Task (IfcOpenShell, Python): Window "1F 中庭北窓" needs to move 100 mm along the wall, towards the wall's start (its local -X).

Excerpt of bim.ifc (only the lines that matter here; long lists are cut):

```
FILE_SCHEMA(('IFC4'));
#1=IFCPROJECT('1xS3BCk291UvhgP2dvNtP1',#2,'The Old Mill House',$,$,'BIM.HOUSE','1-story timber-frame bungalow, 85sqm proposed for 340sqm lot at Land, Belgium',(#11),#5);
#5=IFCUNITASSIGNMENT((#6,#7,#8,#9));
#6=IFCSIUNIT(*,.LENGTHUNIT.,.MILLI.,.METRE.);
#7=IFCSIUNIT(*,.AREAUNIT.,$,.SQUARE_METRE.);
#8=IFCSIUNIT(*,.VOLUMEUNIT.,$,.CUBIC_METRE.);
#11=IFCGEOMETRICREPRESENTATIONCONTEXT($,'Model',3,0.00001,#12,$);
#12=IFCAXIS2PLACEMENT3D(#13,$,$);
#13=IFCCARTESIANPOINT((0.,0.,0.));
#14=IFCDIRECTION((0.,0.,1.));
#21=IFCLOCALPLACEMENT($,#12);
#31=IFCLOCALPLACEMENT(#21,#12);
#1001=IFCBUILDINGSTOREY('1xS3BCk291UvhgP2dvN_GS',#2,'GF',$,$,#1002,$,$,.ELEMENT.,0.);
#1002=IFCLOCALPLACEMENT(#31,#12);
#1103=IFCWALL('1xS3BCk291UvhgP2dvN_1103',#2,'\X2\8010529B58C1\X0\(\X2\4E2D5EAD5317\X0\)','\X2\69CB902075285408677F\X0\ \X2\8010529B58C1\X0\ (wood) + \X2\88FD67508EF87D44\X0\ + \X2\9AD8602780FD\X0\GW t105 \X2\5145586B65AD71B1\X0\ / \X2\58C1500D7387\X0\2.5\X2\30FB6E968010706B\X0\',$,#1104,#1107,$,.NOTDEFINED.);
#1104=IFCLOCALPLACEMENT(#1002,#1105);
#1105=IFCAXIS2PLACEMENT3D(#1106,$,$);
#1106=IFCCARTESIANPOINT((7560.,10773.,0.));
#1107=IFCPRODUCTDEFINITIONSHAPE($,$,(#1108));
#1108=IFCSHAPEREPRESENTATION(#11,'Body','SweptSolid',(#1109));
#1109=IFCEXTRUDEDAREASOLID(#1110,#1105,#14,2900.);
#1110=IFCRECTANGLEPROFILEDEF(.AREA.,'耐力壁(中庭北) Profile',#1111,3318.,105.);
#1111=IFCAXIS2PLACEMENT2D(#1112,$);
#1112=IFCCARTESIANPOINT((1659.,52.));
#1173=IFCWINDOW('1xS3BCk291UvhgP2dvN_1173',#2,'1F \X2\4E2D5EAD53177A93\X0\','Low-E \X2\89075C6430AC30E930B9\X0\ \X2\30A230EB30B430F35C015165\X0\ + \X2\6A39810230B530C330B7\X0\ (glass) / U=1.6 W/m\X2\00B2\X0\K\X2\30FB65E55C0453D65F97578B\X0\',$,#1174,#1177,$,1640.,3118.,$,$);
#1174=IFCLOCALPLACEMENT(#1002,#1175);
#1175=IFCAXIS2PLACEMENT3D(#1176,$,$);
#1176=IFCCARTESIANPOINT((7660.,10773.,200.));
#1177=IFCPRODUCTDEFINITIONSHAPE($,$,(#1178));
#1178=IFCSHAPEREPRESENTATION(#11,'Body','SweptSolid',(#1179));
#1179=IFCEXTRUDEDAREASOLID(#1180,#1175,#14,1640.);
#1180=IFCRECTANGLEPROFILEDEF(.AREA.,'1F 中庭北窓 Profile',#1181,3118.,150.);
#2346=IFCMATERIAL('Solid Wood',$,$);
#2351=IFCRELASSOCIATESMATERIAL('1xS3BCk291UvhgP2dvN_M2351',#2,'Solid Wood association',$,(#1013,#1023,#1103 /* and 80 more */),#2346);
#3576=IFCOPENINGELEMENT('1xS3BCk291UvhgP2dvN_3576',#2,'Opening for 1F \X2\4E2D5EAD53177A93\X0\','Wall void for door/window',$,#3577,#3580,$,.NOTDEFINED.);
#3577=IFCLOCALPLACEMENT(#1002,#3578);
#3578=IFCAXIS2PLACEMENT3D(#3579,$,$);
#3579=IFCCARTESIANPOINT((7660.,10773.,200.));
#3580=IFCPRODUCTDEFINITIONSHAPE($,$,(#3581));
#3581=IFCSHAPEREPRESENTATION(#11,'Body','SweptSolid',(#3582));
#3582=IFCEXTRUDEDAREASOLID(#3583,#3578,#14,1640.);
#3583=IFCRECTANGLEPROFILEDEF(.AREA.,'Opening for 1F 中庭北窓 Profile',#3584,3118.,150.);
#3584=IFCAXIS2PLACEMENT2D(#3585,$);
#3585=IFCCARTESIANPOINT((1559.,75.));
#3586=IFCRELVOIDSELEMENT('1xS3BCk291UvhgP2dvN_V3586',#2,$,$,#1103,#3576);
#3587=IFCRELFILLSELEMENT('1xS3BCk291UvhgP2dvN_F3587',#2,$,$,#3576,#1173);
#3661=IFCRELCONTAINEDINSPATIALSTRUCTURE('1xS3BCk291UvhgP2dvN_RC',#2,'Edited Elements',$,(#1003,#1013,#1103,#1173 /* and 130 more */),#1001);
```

```python
import ifcopenshell
import ifcopenshell.api.geometry
import ifcopenshell.util.placement
import ifcopenshell.util.unit

model = ifcopenshell.open("bim.ifc")
unit_scale = ifcopenshell.util.unit.calculate_unit_scale(model)

window = model.by_id(1173)
opening = window.FillsVoids[0].RelatingOpeningElement
wall = opening.VoidsElements[0].RelatingBuildingElement

wall_matrix = ifcopenshell.util.placement.get_local_placement(wall.ObjectPlacement)
shift = wall_matrix[:3, 0] * -0.1 / unit_scale
before = ifcopenshell.util.placement.get_local_placement(window.ObjectPlacement)[:3, 3].copy()

# The window is not placed relative to its opening, so move both.
for product in (opening, window):
    matrix = ifcopenshell.util.placement.get_local_placement(product.ObjectPlacement)
    matrix[:3, 3] += shift
    ifcopenshell.api.geometry.edit_object_placement(model, product=product, matrix=matrix, is_si=False)

after = ifcopenshell.util.placement.get_local_placement(window.ObjectPlacement)[:3, 3]
print("window moved by", (after - before).round(3) + 0.0)

model.write("bim_rev.ifc")
```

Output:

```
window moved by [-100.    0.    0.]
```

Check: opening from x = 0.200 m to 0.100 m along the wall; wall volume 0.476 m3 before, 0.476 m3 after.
